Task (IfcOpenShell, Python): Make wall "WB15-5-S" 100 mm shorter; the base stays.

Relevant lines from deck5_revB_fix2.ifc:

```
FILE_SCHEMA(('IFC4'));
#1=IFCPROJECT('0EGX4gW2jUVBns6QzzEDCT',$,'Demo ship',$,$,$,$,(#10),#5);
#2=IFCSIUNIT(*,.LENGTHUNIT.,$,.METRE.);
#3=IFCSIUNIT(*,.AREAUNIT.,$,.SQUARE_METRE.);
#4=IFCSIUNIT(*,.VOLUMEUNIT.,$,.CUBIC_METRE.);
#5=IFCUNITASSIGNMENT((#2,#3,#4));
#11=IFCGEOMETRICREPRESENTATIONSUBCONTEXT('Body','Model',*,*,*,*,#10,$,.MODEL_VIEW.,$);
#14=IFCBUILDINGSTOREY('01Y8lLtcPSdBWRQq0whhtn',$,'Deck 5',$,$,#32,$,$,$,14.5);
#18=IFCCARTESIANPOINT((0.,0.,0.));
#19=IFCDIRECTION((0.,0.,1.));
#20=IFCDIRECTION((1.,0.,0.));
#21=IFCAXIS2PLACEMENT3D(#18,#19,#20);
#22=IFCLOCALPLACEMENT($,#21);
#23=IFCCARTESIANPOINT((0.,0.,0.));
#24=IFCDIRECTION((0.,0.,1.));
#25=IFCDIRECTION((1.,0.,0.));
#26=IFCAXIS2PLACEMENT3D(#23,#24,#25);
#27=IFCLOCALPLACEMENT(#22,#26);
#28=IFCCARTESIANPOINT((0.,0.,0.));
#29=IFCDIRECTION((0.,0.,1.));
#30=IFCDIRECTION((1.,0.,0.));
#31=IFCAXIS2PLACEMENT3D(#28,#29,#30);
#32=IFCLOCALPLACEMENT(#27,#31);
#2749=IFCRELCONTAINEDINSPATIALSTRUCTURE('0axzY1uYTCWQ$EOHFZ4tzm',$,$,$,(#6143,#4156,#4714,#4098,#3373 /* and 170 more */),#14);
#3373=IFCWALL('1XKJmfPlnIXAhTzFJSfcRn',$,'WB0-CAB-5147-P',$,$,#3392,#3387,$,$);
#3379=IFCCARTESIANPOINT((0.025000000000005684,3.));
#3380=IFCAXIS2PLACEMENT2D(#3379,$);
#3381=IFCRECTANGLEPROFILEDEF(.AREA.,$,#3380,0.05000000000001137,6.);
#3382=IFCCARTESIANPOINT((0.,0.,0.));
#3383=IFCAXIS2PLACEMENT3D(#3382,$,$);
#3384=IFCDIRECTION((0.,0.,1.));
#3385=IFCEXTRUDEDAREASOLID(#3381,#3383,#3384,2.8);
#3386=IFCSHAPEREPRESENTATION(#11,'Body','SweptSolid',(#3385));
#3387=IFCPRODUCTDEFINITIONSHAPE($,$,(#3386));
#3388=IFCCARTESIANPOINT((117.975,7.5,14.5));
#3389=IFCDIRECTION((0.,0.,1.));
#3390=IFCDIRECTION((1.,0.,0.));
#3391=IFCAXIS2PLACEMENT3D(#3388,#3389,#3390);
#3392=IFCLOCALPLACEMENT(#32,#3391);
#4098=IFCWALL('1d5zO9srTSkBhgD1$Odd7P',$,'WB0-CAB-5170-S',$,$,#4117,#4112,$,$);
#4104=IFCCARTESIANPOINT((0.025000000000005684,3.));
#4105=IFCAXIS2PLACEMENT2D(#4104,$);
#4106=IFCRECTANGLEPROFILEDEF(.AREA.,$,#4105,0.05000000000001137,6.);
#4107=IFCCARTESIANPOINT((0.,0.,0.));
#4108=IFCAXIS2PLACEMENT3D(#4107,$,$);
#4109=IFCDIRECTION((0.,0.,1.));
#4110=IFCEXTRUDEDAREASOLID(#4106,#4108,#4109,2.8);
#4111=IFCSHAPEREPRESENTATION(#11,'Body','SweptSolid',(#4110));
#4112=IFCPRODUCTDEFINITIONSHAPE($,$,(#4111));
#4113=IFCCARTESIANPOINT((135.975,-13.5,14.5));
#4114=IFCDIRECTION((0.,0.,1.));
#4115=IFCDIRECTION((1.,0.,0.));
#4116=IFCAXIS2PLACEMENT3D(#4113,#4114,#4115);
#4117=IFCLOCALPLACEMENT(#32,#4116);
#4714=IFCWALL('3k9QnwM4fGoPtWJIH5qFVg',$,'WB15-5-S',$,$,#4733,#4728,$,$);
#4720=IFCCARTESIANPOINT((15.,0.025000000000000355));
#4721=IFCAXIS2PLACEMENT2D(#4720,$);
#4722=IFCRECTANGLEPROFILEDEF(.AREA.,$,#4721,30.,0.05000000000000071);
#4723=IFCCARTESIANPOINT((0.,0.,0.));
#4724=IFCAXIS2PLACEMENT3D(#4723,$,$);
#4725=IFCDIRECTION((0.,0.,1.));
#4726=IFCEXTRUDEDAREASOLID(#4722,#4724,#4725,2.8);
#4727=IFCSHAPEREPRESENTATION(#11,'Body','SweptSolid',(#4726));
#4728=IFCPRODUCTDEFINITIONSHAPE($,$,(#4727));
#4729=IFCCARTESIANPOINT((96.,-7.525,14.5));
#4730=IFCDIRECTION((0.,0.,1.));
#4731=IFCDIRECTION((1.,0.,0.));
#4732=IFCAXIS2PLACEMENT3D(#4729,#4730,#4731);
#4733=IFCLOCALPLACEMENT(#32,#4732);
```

```python
import ifcopenshell
import ifcopenshell.geom
import ifcopenshell.util.representation
import ifcopenshell.util.shape

model = ifcopenshell.open("deck5_revB_fix2.ifc")
settings = ifcopenshell.geom.settings()


def volume(element):
    """Net volume in cubic metres, openings subtracted."""
    shape = ifcopenshell.geom.create_shape(settings, element)
    return ifcopenshell.util.shape.get_volume(shape.geometry)


wall = model.by_guid("3k9QnwM4fGoPtWJIH5qFVg")
before = volume(wall)

body = ifcopenshell.util.representation.get_representation(wall, "Model", "Body")
solid = body.Items[0]
old_height = solid.Depth
solid.Depth -= 0.1
after = volume(wall)

print(f"height {old_height:g} -> {solid.Depth:g}, volume {before:.3f} -> {after:.3f} m3")

model.write("deck5_revB_fix2_edited.ifc")
```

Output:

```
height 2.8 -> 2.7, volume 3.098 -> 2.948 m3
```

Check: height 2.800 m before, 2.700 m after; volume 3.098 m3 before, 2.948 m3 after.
